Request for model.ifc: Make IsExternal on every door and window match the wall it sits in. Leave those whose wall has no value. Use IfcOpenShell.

First a look at what the model holds.

```python
import ifcopenshell
import ifcopenshell.util.element

model = ifcopenshell.open("model.ifc")
print(model.schema)
seen = {}
for e in model.by_type("IfcDoor") + model.by_type("IfcWindow"):
    if not e.FillsVoids:
        continue
    host = e.FillsVoids[0].RelatingOpeningElement.VoidsElements[0].RelatingBuildingElement
    own = ifcopenshell.util.element.get_pset(e, f"Pset_{e.is_a()[3:].removesuffix('StandardCase')}Common", "IsExternal")
    wall = ifcopenshell.util.element.get_pset(host, "Pset_WallCommon", "IsExternal")
    seen[e.is_a(), own, wall] = seen.get((e.is_a(), own, wall), 0) + 1
for (cls, own, wall), count in sorted(seen.items(), key=str):
    print(count, cls, "IsExternal:", own, "| host wall:", wall)
```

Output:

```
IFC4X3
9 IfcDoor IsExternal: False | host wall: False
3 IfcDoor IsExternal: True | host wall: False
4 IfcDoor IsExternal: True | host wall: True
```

```python
import ifcopenshell
import ifcopenshell.api.pset
import ifcopenshell.util.element

model = ifcopenshell.open("model.ifc")

count = 0
for ifc_class, pset_name in (("IfcDoor", "Pset_DoorCommon"), ("IfcWindow", "Pset_WindowCommon")):
    for e in model.by_type(ifc_class):
        if not e.FillsVoids:
            continue
        host = e.FillsVoids[0].RelatingOpeningElement.VoidsElements[0].RelatingBuildingElement
        external = ifcopenshell.util.element.get_pset(host, "Pset_WallCommon", "IsExternal")
        if external is None or ifcopenshell.util.element.get_pset(e, pset_name, "IsExternal") == external:
            continue
        pset = ifcopenshell.api.pset.add_pset(model, product=e, name=pset_name)
        ifcopenshell.api.pset.edit_pset(model, pset=pset, properties={"IsExternal": external})
        count += 1

print(count, "updated")

model.write("model_v2.ifc")
```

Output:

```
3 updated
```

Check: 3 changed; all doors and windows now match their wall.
